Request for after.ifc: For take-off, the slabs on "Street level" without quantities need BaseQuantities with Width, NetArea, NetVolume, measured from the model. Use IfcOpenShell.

First a look at what the model holds.

```python
import ifcopenshell
import ifcopenshell.util.element
import ifcopenshell.util.unit

model = ifcopenshell.open("after.ifc")
print(model.schema)
for unit_type in ("LENGTHUNIT", "AREAUNIT", "VOLUMEUNIT"):
    print(unit_type, ifcopenshell.util.unit.calculate_unit_scale(model, unit_type))
storey = next(s for s in model.by_type("IfcBuildingStorey") if s.Name == "Street level")
slabs = [e for e in ifcopenshell.util.element.get_decomposition(storey) if e.is_a("IfcSlab")]
for e in sorted(slabs, key=lambda e: e.id()):
    print(e.id(), e.is_a(), e.Name, list(ifcopenshell.util.element.get_psets(e, qtos_only=True)), sep=" | ")
```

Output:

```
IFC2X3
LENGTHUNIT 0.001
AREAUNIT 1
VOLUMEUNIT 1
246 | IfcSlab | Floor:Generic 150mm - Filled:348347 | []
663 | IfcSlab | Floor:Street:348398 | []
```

```python
import ifcopenshell
import ifcopenshell.api.pset
import ifcopenshell.geom
import ifcopenshell.util.element
import ifcopenshell.util.shape
import ifcopenshell.util.unit

model = ifcopenshell.open("after.ifc")
unit_scale = ifcopenshell.util.unit.calculate_unit_scale(model)
area_scale = ifcopenshell.util.unit.calculate_unit_scale(model, "AREAUNIT")
volume_scale = ifcopenshell.util.unit.calculate_unit_scale(model, "VOLUMEUNIT")
settings = ifcopenshell.geom.settings()

storey = next(s for s in model.by_type("IfcBuildingStorey") if s.Name == "Street level")
slabs = [e for e in ifcopenshell.util.element.get_decomposition(storey) if e.is_a("IfcSlab")]

for e in sorted(slabs, key=lambda e: e.id()):
    if ifcopenshell.util.element.get_psets(e, qtos_only=True, should_inherit=False):
        continue
    # Geometry comes back in metres, in the element's own axes.
    shape = ifcopenshell.geom.create_shape(settings, e)
    values = {
        "Width": ifcopenshell.util.shape.get_z(shape.geometry) / unit_scale,
        "NetArea": ifcopenshell.util.shape.get_footprint_area(shape.geometry) / area_scale,
        "NetVolume": ifcopenshell.util.shape.get_volume(shape.geometry) / volume_scale,
    }
    qto = ifcopenshell.api.pset.add_qto(model, product=e, name="BaseQuantities")
    ifcopenshell.api.pset.edit_qto(model, qto=qto, properties=values)
    print(e.id(), {k: round(v, 3) for k, v in values.items()})

model.write("after_updated.ifc")
```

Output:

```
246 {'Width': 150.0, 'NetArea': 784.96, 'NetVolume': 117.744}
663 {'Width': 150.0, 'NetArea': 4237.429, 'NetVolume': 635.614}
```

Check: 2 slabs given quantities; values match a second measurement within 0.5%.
